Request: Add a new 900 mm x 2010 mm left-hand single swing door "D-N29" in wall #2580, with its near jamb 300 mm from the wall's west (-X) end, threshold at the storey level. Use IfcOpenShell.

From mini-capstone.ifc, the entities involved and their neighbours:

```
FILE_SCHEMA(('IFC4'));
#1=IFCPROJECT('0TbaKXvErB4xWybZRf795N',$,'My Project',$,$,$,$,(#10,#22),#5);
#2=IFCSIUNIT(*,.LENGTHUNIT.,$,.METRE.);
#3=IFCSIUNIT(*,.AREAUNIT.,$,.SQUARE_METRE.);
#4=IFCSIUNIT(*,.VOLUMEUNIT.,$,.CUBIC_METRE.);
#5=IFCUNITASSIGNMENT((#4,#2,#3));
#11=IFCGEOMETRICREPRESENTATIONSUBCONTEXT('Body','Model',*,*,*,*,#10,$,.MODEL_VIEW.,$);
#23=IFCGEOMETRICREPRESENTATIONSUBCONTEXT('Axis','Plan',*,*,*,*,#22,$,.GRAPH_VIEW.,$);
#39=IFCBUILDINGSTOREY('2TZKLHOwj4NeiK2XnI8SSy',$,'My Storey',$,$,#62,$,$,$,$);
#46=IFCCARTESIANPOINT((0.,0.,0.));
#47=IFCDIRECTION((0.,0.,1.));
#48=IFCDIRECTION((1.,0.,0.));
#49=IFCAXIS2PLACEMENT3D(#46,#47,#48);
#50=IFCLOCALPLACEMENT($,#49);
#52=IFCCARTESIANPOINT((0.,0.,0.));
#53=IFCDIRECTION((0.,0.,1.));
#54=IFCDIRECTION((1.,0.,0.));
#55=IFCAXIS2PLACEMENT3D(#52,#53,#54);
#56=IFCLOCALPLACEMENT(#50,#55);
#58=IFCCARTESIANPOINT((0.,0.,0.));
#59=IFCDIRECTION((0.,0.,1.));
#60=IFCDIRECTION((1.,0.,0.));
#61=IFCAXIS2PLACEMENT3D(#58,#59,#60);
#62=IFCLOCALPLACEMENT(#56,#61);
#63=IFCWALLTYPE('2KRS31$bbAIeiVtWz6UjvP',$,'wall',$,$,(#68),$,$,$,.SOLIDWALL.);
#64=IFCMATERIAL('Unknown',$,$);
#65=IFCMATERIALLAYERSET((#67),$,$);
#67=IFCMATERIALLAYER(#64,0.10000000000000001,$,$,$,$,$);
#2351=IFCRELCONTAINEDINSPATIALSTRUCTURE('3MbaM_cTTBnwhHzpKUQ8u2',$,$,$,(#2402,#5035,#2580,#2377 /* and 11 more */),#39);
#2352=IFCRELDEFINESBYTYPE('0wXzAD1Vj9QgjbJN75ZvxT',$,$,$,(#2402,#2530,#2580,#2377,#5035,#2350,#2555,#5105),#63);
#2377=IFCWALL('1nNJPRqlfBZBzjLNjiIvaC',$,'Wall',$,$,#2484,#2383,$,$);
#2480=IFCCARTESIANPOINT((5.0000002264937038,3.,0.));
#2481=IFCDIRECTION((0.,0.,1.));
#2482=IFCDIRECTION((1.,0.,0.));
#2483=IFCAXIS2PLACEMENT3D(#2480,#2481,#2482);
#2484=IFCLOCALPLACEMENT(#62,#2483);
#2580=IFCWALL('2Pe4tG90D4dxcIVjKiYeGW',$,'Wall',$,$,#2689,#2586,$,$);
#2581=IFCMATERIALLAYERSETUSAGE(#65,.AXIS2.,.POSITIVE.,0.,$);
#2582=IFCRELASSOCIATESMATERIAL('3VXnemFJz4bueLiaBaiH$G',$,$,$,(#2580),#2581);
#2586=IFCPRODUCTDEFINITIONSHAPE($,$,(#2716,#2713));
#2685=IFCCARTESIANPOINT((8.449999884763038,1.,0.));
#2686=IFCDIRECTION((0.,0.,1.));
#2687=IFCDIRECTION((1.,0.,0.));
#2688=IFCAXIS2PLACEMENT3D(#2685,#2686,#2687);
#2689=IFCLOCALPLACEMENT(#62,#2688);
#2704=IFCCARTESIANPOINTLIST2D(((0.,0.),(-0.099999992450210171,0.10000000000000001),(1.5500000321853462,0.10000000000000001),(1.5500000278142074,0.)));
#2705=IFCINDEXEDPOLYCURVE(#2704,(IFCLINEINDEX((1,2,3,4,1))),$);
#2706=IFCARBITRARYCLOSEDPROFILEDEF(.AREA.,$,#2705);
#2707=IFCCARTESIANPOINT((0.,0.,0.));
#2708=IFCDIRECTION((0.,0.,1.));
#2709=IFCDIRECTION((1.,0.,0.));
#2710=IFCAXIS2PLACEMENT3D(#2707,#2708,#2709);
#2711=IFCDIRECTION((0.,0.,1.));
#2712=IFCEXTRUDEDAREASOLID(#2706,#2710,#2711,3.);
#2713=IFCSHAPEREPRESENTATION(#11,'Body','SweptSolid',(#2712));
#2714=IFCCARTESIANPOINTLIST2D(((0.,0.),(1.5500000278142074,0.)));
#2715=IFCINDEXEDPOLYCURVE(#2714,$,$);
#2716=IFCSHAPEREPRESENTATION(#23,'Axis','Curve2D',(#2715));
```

```python
import numpy as np
import ifcopenshell
import ifcopenshell.api.feature
import ifcopenshell.api.geometry
import ifcopenshell.api.root
import ifcopenshell.api.spatial
import ifcopenshell.geom
import ifcopenshell.util.element
import ifcopenshell.util.placement
import ifcopenshell.util.representation
import ifcopenshell.util.shape
import ifcopenshell.util.unit

model = ifcopenshell.open("mini-capstone.ifc")
unit_scale = ifcopenshell.util.unit.calculate_unit_scale(model)
settings = ifcopenshell.geom.settings()


def volume(element):
    """Net volume in cubic metres, openings subtracted."""
    shape = ifcopenshell.geom.create_shape(settings, element)
    return ifcopenshell.util.shape.get_volume(shape.geometry)


wall = model.by_guid("2Pe4tG90D4dxcIVjKiYeGW")
storey = ifcopenshell.util.element.get_container(wall, ifc_class="IfcBuildingStorey")
context = ifcopenshell.util.representation.get_context(model, "Model", "Body", "MODEL_VIEW")
before = volume(wall)

width, height, from_end, sill = 0.9, 2.01, 0.3, 0.0  # metres

# The wall runs along its own X axis, and the end named is its -X end.
wall_shape = ifcopenshell.geom.create_shape(settings, wall)
x, y, z = ifcopenshell.util.shape.get_vertices(wall_shape.geometry).T
start = x.min() + from_end
face, thickness = float(y.min()), float(y.max() - y.min())
wall_matrix = ifcopenshell.util.placement.get_local_placement(wall.ObjectPlacement)
level = ifcopenshell.util.placement.get_local_placement(storey.ObjectPlacement)[2, 3]


def in_wall(x, y):
    """Placement at x, y metres in the wall's axes, at sill height."""
    matrix = wall_matrix.copy()
    matrix[:, 3] = wall_matrix @ np.array([x / unit_scale, y / unit_scale, 0.0, 1.0])
    matrix[2, 3] = level + sill / unit_scale
    return matrix


# Opening: a box that overshoots both wall faces by 50 mm.
opening = ifcopenshell.api.root.create_entity(model, ifc_class="IfcOpeningElement", predefined_type="OPENING")
box = ifcopenshell.api.geometry.add_wall_representation(
    model, context=context, length=width, height=height, thickness=thickness + 0.1
)
ifcopenshell.api.geometry.assign_representation(model, product=opening, representation=box)
ifcopenshell.api.geometry.edit_object_placement(model, product=opening, matrix=in_wall(start, face - 0.05), is_si=False)
ifcopenshell.api.feature.add_feature(model, feature=opening, element=wall)

door = ifcopenshell.api.root.create_entity(model, ifc_class="IfcDoor", name="D-N29", predefined_type="DOOR")
door.OverallWidth, door.OverallHeight = width / unit_scale, height / unit_scale
door.OperationType = "SINGLE_SWING_LEFT"
body = ifcopenshell.api.geometry.add_door_representation(
    model,
    context=context,
    overall_width=door.OverallWidth,
    overall_height=door.OverallHeight,
    operation_type="SINGLE_SWING_LEFT",
    lining_properties={"LiningDepth": thickness / unit_scale, "ThresholdDepth": thickness / unit_scale},
)
ifcopenshell.api.geometry.assign_representation(model, product=door, representation=body)
ifcopenshell.api.spatial.assign_container(model, products=[door], relating_structure=storey)
ifcopenshell.api.feature.add_filling(model, opening=opening, element=door)

# The lining spans the wall, so the door starts at the wall face.
ifcopenshell.api.geometry.edit_object_placement(model, product=door, matrix=in_wall(start, face), is_si=False)

after = volume(wall)

print(f"wall volume {before:.3f} -> {after:.3f} m3")

model.write("mini-capstone-out.ifc")
```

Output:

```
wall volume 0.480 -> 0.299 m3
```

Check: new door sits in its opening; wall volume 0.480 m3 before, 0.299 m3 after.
